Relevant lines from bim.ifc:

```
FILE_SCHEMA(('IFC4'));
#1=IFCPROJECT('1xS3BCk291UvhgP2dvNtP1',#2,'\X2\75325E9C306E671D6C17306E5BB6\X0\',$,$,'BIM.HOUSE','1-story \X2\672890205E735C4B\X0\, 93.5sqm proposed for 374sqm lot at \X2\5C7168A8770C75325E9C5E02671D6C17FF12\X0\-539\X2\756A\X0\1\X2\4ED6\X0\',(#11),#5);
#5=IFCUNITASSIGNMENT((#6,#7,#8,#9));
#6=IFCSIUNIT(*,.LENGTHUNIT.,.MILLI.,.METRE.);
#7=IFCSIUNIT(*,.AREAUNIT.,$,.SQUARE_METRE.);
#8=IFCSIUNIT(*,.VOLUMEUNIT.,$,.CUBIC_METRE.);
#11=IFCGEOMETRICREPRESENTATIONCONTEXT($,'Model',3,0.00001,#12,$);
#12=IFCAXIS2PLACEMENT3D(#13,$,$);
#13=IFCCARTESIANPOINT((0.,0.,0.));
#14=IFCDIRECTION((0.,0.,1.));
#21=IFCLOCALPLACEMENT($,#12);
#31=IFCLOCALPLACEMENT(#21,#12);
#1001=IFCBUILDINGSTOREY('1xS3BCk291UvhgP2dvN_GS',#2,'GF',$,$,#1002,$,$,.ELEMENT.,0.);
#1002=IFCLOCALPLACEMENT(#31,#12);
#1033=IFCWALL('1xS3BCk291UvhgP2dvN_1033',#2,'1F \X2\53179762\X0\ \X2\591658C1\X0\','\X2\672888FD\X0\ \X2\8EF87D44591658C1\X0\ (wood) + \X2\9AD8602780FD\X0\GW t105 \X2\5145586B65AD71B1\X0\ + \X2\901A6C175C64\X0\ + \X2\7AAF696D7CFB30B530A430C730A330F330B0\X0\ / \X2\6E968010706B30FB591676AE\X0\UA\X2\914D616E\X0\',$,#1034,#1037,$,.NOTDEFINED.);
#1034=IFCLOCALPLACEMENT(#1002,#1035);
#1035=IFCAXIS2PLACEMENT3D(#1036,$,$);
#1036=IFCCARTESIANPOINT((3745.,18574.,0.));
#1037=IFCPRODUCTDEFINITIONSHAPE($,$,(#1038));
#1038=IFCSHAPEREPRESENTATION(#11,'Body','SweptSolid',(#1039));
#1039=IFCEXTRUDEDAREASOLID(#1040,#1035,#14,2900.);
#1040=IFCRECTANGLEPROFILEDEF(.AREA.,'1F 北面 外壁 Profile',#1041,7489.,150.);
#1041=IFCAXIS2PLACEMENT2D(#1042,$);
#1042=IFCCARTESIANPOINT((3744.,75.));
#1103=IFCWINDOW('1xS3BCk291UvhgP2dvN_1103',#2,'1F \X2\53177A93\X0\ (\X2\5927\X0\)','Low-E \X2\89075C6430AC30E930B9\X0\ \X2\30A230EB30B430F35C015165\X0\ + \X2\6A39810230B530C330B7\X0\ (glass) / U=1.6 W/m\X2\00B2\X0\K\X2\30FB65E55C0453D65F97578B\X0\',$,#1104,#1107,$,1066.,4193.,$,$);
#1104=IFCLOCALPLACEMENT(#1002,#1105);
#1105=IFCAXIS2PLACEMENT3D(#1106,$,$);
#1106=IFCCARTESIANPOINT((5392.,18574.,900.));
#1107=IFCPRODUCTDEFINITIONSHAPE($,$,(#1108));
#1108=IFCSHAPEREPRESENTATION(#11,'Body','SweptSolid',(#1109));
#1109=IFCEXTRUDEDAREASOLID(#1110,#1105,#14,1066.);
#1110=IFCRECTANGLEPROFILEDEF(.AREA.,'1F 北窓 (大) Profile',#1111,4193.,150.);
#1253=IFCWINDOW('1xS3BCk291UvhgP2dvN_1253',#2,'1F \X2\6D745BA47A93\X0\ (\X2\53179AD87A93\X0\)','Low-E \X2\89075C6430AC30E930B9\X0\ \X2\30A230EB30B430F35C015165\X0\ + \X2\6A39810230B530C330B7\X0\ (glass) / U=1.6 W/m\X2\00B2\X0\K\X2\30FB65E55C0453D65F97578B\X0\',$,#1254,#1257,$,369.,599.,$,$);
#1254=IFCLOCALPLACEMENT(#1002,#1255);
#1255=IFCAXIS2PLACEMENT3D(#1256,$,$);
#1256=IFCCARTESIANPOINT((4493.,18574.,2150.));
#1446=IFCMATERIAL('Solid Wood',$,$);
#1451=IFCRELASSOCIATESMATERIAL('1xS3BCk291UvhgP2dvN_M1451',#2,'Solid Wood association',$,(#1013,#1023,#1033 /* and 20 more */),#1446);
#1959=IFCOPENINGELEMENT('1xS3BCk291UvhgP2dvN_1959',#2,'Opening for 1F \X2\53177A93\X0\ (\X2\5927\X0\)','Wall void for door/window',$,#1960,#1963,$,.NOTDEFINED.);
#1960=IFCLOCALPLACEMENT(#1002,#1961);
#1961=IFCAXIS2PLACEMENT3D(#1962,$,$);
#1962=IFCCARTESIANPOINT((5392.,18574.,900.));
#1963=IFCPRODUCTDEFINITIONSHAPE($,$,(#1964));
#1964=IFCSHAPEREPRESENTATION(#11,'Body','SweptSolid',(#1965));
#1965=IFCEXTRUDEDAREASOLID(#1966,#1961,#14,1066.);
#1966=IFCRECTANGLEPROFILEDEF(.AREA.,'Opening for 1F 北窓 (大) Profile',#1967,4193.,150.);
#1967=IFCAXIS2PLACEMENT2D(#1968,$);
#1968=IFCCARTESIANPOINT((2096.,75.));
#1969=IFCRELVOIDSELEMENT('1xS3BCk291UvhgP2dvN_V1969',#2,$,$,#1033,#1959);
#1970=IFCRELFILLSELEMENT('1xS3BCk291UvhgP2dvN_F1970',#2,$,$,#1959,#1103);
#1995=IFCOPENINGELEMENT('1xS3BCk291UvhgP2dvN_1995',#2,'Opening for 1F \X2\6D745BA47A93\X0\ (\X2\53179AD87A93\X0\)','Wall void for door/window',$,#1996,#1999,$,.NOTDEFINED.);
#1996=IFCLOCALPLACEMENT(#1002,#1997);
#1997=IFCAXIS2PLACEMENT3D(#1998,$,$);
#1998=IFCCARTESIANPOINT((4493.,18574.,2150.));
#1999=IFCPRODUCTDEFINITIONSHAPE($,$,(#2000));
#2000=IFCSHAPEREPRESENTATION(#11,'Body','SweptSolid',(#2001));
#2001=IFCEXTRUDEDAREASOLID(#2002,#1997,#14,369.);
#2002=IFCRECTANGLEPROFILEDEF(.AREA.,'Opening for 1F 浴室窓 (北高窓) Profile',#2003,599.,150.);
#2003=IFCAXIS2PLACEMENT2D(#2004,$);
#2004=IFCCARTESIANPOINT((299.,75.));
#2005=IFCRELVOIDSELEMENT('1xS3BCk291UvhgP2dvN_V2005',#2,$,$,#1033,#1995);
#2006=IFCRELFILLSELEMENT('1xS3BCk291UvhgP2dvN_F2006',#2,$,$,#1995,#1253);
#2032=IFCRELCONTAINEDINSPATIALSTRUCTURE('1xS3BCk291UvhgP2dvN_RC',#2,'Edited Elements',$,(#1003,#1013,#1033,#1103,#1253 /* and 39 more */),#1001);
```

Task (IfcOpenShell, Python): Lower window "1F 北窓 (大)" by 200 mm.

```python
import numpy as np
import ifcopenshell
import ifcopenshell.api.geometry
import ifcopenshell.util.placement
import ifcopenshell.util.unit

model = ifcopenshell.open("bim.ifc")
unit_scale = ifcopenshell.util.unit.calculate_unit_scale(model)

window = model.by_guid("1xS3BCk291UvhgP2dvN_1103")
opening = window.FillsVoids[0].RelatingOpeningElement
dz = -0.2 / unit_scale

shift = np.array([0.0, 0.0, dz])
# The window is not placed relative to its opening, so move both.
for product in (opening, window):
    matrix = ifcopenshell.util.placement.get_local_placement(product.ObjectPlacement)
    matrix[:3, 3] += shift
    ifcopenshell.api.geometry.edit_object_placement(model, product=product, matrix=matrix, is_si=False)

print(f"moved by {dz * unit_scale:+.3f} m")

model.write("bim_updated.ifc")
```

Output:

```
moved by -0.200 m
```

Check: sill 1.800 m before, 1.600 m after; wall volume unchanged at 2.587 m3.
